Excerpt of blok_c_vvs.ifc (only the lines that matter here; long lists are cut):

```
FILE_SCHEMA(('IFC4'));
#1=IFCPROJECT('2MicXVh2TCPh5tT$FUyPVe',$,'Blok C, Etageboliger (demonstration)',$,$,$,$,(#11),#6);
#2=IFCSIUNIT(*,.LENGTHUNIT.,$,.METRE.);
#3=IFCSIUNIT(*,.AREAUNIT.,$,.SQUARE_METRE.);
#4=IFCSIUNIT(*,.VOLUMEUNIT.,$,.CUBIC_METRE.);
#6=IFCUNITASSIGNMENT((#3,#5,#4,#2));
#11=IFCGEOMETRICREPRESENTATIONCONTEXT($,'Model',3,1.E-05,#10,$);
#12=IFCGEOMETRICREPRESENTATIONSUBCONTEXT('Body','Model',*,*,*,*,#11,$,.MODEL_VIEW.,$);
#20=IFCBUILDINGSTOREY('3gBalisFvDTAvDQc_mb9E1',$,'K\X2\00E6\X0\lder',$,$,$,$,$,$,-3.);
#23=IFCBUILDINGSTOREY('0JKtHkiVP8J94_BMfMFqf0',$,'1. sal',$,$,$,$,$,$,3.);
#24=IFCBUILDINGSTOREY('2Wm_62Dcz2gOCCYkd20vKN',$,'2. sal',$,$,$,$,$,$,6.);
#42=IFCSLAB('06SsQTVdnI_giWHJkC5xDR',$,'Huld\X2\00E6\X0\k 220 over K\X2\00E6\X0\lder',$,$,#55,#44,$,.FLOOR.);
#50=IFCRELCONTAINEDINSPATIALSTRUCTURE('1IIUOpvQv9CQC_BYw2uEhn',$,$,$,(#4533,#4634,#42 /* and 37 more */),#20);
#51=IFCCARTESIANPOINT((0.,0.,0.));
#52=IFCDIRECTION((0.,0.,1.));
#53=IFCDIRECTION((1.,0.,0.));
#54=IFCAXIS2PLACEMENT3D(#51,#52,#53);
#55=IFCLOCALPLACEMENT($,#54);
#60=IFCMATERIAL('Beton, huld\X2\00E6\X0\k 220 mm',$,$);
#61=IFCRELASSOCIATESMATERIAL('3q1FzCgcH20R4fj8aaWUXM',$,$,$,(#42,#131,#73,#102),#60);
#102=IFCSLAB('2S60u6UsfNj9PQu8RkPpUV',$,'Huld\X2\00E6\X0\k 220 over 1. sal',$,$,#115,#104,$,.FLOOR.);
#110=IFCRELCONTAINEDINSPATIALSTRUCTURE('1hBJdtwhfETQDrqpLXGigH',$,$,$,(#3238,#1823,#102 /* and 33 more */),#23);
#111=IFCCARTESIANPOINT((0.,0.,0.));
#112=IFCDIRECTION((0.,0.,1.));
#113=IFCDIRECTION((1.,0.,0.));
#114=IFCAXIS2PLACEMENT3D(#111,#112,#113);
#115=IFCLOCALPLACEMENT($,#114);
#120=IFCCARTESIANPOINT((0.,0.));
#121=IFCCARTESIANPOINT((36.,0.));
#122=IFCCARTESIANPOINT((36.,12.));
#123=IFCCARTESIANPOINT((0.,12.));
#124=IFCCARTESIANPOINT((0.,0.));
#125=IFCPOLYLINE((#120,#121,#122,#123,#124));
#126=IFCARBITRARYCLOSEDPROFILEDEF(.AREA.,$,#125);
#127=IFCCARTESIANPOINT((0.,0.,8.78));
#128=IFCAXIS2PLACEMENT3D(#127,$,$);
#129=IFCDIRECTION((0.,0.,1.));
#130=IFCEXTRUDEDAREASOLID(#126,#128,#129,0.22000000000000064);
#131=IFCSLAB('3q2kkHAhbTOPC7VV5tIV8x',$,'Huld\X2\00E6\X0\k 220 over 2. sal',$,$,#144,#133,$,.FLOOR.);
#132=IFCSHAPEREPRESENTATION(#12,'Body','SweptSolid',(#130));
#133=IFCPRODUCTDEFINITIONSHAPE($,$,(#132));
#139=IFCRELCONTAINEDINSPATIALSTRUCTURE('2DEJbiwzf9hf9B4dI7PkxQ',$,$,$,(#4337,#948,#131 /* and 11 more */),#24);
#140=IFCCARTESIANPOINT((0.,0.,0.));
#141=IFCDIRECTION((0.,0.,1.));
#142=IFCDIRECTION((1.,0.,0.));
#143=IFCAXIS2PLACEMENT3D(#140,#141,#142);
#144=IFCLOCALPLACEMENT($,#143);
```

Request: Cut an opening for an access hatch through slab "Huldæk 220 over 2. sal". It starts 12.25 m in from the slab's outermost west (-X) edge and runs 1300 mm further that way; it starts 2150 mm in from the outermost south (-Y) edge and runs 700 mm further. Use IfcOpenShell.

```python
import numpy as np
import ifcopenshell
import ifcopenshell.api.feature
import ifcopenshell.api.geometry
import ifcopenshell.api.root
import ifcopenshell.geom
import ifcopenshell.util.placement
import ifcopenshell.util.representation
import ifcopenshell.util.shape
import ifcopenshell.util.unit

model = ifcopenshell.open("blok_c_vvs.ifc")
unit_scale = ifcopenshell.util.unit.calculate_unit_scale(model)
settings = ifcopenshell.geom.settings()


def volume(element):
    """Net volume in cubic metres, openings subtracted."""
    shape = ifcopenshell.geom.create_shape(settings, element)
    return ifcopenshell.util.shape.get_volume(shape.geometry)


slab = model.by_guid("3q2kkHAhbTOPC7VV5tIV8x")
before = volume(slab)

# Extent in the slab's own axes, in metres. The edges named are its -X and -Y sides.
slab_shape = ifcopenshell.geom.create_shape(settings, slab)
vertices = ifcopenshell.util.shape.get_vertices(slab_shape.geometry)
x_min, y_min, bottom = vertices.min(axis=0)
top = vertices[:, 2].max()

opening = ifcopenshell.api.root.create_entity(model, ifc_class="IfcOpeningElement", name="Access hatch opening", predefined_type="OPENING")
context = ifcopenshell.util.representation.get_context(model, "Model", "Body", "MODEL_VIEW")
width, depth = 1.3, 0.7
outline = [(0.0, 0.0), (width, 0.0), (width, depth), (0.0, depth), (0.0, 0.0)]
# Overshoot both faces by 50 mm so the cut is clean.
shape = ifcopenshell.api.geometry.add_slab_representation(
    model, context=context, depth=top - bottom + 0.1, polyline=outline
)
ifcopenshell.api.geometry.assign_representation(model, product=opening, representation=shape)

matrix = ifcopenshell.util.placement.get_local_placement(slab.ObjectPlacement)
matrix[:, 3] = matrix @ np.append(np.array([x_min + 12.25, y_min + 2.15, bottom - 0.05]) / unit_scale, 1.0)
ifcopenshell.api.geometry.edit_object_placement(model, product=opening, matrix=matrix, is_si=False)
ifcopenshell.api.feature.add_feature(model, feature=opening, element=slab)

after = volume(slab)

print(f"slab volume {before:.3f} -> {after:.3f} m3")

model.write("blok_c_vvs_updated.ifc")
```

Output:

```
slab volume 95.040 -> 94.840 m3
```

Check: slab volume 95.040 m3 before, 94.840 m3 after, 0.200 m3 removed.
